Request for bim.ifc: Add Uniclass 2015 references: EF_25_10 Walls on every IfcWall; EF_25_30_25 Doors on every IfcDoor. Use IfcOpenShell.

First a look at what the model holds.

```python
import ifcopenshell

model = ifcopenshell.open("bim.ifc")
print(model.schema)
print("classifications:", [c.Name for c in model.by_type("IfcClassification")])
for ifc_class in ("IfcDoor", "IfcRoof", "IfcStair", "IfcWall", "IfcWindow"):
    print(ifc_class, len(model.by_type(ifc_class)))
```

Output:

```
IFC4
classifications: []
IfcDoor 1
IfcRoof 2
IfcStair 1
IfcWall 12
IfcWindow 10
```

```python
import ifcopenshell
import ifcopenshell.api.classification

model = ifcopenshell.open("bim.ifc")

system = ifcopenshell.api.classification.add_classification(model, classification="Uniclass 2015")

codes = {
    "IfcWall": ("EF_25_10", "Walls"),
    "IfcDoor": ("EF_25_30_25", "Doors"),
}
for ifc_class, (code, name) in codes.items():
    products = model.by_type(ifc_class)
    ifcopenshell.api.classification.add_reference(
        model, products=products, classification=system, identification=code, name=name
    )
    print(code, len(products))

model.write("bim_edited.ifc")
```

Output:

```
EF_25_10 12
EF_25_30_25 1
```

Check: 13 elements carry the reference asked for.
